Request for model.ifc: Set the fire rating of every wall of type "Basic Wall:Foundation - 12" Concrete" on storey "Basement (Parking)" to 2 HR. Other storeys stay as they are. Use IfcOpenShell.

First a look at what the model holds.

```python
import ifcopenshell
import ifcopenshell.util.element

model = ifcopenshell.open("model.ifc")
print(model.schema)
storey = next(s for s in model.by_type("IfcBuildingStorey") if s.Name == "Basement (Parking)")
walls = [e for e in ifcopenshell.util.element.get_decomposition(storey) if e.is_a("IfcWall")]
seen = {}
for e in walls:
    element_type = ifcopenshell.util.element.get_type(e)
    key = (element_type.Name if element_type != e and element_type else None, ifcopenshell.util.element.get_pset(e, "Pset_WallCommon", "FireRating"))
    seen[key] = seen.get(key, 0) + 1
for (name, value), count in sorted(seen.items(), key=str):
    print(count, "x", name, "|", value)
```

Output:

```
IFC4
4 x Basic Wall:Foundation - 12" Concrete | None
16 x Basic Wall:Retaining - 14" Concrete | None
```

```python
import ifcopenshell
import ifcopenshell.api.pset
import ifcopenshell.util.element

model = ifcopenshell.open("model.ifc")

storey = next(s for s in model.by_type("IfcBuildingStorey") if s.Name == "Basement (Parking)")
walls = [e for e in ifcopenshell.util.element.get_decomposition(storey) if e.is_a("IfcWall")]

count = 0
for e in walls:
    element_type = ifcopenshell.util.element.get_type(e)
    if element_type in (None, e) or element_type.Name != 'Basic Wall:Foundation - 12" Concrete':
        continue
    # add_pset returns the element's existing set when there is one.
    pset = ifcopenshell.api.pset.add_pset(model, product=e, name="Pset_WallCommon")
    ifcopenshell.api.pset.edit_pset(model, pset=pset, properties={"FireRating": "2 HR"})
    count += 1

print(count, "walls updated")

model.write("model_updated.ifc")
```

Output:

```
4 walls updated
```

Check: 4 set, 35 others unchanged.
